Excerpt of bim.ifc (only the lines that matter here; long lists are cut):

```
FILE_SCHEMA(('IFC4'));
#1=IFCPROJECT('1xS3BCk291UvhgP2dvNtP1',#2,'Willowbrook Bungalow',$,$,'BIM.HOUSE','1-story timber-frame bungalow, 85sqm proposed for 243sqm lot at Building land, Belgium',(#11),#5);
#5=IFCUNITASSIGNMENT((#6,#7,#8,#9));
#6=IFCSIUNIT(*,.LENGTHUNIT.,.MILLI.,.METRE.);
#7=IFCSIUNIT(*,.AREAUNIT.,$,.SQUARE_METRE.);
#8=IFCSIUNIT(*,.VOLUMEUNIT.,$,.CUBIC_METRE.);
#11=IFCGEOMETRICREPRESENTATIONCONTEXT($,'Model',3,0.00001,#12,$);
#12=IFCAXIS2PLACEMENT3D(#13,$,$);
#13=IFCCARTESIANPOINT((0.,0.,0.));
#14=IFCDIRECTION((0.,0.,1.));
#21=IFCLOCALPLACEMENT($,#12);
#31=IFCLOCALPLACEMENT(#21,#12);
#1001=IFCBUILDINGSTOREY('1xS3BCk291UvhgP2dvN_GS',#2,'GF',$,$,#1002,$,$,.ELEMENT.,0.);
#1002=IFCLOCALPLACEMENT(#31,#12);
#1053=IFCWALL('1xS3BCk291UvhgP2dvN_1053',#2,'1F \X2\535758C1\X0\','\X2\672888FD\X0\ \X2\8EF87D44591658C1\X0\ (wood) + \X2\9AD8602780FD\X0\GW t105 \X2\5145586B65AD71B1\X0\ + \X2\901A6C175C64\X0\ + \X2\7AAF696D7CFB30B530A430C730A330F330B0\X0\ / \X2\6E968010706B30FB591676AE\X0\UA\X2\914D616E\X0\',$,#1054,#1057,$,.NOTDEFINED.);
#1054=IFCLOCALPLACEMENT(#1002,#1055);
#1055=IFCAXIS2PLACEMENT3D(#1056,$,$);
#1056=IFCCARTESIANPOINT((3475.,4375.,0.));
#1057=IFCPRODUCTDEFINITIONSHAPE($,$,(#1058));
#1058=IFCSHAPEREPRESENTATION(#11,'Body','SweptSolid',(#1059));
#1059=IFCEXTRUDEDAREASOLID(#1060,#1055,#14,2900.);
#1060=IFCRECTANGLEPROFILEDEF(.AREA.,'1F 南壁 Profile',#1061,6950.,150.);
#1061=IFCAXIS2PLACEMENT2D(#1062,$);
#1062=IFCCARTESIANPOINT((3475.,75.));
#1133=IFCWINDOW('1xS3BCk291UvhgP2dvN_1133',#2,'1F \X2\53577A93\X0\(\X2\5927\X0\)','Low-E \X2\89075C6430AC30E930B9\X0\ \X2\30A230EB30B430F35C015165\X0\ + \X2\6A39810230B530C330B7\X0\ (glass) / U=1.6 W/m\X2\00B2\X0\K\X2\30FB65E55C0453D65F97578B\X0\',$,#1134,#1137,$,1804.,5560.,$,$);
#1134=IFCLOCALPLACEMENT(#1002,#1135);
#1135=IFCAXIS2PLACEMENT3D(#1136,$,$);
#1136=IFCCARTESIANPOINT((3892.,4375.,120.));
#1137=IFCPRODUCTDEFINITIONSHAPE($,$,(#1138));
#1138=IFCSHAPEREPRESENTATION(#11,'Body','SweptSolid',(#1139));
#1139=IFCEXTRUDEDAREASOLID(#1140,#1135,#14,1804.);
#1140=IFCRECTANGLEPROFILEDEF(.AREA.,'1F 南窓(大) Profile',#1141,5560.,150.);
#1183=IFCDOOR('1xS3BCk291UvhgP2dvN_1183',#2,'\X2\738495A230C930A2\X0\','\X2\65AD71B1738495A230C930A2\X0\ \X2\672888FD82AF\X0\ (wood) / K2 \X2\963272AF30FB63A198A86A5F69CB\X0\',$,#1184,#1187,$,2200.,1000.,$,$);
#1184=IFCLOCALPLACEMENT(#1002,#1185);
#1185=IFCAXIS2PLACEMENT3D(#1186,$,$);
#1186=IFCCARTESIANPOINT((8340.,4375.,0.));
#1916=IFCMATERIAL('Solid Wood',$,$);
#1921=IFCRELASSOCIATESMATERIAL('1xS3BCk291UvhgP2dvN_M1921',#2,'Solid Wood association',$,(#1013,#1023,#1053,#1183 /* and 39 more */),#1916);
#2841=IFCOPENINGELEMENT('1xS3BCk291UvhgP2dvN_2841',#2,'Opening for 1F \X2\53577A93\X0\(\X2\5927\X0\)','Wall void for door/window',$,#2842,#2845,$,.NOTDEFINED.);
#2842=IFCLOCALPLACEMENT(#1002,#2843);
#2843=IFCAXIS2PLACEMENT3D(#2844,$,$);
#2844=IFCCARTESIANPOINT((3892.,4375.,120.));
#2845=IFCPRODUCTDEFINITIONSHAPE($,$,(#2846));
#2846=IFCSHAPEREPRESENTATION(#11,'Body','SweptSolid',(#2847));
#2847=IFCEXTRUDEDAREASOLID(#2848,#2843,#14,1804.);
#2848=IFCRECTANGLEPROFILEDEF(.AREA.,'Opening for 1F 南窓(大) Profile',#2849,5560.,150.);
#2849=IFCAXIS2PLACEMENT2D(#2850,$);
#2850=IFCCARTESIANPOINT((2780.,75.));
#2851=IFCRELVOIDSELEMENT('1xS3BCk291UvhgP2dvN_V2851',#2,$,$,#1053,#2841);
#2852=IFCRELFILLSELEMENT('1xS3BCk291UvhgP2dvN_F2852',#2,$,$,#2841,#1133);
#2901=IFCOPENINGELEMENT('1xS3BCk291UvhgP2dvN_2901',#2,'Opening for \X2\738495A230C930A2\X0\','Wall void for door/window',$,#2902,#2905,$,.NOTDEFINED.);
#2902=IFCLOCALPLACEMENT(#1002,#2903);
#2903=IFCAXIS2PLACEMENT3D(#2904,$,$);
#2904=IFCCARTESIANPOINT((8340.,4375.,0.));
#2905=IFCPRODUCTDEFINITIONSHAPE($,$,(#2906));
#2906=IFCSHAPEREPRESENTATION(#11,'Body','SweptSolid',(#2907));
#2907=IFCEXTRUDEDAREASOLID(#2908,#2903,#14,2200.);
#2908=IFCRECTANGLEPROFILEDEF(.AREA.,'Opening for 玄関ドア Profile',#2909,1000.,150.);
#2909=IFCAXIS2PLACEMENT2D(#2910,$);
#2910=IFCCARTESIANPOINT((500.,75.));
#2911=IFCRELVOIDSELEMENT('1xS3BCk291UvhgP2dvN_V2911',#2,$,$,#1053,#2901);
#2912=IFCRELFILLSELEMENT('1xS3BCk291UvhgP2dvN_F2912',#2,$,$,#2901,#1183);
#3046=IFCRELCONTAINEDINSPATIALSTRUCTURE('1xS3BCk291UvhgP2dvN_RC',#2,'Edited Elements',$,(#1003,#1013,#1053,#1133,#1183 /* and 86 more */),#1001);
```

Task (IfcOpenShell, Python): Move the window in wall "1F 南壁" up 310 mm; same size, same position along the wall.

```python
import numpy as np
import ifcopenshell
import ifcopenshell.api.geometry
import ifcopenshell.util.placement
import ifcopenshell.util.unit

model = ifcopenshell.open("bim.ifc")
unit_scale = ifcopenshell.util.unit.calculate_unit_scale(model)

window = model.by_guid("1xS3BCk291UvhgP2dvN_1133")
opening = window.FillsVoids[0].RelatingOpeningElement
dz = 310.0

shift = np.array([0.0, 0.0, dz])
# The window is not placed relative to its opening, so move both.
for product in (opening, window):
    matrix = ifcopenshell.util.placement.get_local_placement(product.ObjectPlacement)
    matrix[:3, 3] += shift
    ifcopenshell.api.geometry.edit_object_placement(model, product=product, matrix=matrix, is_si=False)

print(f"moved by {dz * unit_scale:+.3f} m")

model.write("bim_rev.ifc")
```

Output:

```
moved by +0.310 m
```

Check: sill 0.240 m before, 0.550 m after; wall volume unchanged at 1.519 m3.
